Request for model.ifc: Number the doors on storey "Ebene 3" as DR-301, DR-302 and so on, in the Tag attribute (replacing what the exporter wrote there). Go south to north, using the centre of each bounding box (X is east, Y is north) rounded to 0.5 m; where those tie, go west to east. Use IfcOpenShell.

First a look at what the model holds.

```python
import ifcopenshell
import ifcopenshell.util.element
import ifcopenshell.util.placement

model = ifcopenshell.open("model.ifc")
print(model.schema)
storey = next(s for s in model.by_type("IfcBuildingStorey") if s.Name == "Ebene 3")
doors = [e for e in ifcopenshell.util.element.get_decomposition(storey) if e.is_a("IfcDoor")]
for e in sorted(doors, key=lambda e: e.id()):
    origin = ifcopenshell.util.placement.get_local_placement(e.ObjectPlacement)[:3, 3]
    print(e.id(), e.Tag, e.Name, origin.round(2) + 0.0, sep=" | ")
```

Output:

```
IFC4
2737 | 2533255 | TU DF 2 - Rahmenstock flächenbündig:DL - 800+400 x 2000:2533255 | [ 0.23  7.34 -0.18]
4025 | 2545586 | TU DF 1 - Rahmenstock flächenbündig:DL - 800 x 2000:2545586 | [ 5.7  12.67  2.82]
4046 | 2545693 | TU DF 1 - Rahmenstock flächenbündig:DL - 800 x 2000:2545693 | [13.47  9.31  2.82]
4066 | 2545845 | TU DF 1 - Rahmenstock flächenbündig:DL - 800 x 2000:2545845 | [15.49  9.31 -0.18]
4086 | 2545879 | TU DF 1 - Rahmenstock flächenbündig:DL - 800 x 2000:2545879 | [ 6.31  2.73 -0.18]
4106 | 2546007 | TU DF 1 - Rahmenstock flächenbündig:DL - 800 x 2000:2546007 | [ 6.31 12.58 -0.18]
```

```python
import ifcopenshell
import ifcopenshell.geom
import ifcopenshell.util.element
import ifcopenshell.util.shape

model = ifcopenshell.open("model.ifc")
settings = ifcopenshell.geom.settings()
settings.set("use-world-coords", True)


def centre(element):
    shape = ifcopenshell.geom.create_shape(settings, element)
    return ifcopenshell.util.shape.get_bbox_centroid(shape.geometry)


storey = next(s for s in model.by_type("IfcBuildingStorey") if s.Name == "Ebene 3")
doors = [e for e in ifcopenshell.util.element.get_decomposition(storey) if e.is_a("IfcDoor")]

# Insertion points can sit at a corner or the storey origin, so sort by the geometry (in metres).
centres = {e: centre(e) for e in doors}
doors.sort(key=lambda e: (round(centres[e][1] / 0.5), centres[e][0]))

for i, e in enumerate(doors, start=1):
    number = f"DR-3{i:02d}"
    e.Tag = number
    print(e.id(), number)

model.write("model-out.ifc")
```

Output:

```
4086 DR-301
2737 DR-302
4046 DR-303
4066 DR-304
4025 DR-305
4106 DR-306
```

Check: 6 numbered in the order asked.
